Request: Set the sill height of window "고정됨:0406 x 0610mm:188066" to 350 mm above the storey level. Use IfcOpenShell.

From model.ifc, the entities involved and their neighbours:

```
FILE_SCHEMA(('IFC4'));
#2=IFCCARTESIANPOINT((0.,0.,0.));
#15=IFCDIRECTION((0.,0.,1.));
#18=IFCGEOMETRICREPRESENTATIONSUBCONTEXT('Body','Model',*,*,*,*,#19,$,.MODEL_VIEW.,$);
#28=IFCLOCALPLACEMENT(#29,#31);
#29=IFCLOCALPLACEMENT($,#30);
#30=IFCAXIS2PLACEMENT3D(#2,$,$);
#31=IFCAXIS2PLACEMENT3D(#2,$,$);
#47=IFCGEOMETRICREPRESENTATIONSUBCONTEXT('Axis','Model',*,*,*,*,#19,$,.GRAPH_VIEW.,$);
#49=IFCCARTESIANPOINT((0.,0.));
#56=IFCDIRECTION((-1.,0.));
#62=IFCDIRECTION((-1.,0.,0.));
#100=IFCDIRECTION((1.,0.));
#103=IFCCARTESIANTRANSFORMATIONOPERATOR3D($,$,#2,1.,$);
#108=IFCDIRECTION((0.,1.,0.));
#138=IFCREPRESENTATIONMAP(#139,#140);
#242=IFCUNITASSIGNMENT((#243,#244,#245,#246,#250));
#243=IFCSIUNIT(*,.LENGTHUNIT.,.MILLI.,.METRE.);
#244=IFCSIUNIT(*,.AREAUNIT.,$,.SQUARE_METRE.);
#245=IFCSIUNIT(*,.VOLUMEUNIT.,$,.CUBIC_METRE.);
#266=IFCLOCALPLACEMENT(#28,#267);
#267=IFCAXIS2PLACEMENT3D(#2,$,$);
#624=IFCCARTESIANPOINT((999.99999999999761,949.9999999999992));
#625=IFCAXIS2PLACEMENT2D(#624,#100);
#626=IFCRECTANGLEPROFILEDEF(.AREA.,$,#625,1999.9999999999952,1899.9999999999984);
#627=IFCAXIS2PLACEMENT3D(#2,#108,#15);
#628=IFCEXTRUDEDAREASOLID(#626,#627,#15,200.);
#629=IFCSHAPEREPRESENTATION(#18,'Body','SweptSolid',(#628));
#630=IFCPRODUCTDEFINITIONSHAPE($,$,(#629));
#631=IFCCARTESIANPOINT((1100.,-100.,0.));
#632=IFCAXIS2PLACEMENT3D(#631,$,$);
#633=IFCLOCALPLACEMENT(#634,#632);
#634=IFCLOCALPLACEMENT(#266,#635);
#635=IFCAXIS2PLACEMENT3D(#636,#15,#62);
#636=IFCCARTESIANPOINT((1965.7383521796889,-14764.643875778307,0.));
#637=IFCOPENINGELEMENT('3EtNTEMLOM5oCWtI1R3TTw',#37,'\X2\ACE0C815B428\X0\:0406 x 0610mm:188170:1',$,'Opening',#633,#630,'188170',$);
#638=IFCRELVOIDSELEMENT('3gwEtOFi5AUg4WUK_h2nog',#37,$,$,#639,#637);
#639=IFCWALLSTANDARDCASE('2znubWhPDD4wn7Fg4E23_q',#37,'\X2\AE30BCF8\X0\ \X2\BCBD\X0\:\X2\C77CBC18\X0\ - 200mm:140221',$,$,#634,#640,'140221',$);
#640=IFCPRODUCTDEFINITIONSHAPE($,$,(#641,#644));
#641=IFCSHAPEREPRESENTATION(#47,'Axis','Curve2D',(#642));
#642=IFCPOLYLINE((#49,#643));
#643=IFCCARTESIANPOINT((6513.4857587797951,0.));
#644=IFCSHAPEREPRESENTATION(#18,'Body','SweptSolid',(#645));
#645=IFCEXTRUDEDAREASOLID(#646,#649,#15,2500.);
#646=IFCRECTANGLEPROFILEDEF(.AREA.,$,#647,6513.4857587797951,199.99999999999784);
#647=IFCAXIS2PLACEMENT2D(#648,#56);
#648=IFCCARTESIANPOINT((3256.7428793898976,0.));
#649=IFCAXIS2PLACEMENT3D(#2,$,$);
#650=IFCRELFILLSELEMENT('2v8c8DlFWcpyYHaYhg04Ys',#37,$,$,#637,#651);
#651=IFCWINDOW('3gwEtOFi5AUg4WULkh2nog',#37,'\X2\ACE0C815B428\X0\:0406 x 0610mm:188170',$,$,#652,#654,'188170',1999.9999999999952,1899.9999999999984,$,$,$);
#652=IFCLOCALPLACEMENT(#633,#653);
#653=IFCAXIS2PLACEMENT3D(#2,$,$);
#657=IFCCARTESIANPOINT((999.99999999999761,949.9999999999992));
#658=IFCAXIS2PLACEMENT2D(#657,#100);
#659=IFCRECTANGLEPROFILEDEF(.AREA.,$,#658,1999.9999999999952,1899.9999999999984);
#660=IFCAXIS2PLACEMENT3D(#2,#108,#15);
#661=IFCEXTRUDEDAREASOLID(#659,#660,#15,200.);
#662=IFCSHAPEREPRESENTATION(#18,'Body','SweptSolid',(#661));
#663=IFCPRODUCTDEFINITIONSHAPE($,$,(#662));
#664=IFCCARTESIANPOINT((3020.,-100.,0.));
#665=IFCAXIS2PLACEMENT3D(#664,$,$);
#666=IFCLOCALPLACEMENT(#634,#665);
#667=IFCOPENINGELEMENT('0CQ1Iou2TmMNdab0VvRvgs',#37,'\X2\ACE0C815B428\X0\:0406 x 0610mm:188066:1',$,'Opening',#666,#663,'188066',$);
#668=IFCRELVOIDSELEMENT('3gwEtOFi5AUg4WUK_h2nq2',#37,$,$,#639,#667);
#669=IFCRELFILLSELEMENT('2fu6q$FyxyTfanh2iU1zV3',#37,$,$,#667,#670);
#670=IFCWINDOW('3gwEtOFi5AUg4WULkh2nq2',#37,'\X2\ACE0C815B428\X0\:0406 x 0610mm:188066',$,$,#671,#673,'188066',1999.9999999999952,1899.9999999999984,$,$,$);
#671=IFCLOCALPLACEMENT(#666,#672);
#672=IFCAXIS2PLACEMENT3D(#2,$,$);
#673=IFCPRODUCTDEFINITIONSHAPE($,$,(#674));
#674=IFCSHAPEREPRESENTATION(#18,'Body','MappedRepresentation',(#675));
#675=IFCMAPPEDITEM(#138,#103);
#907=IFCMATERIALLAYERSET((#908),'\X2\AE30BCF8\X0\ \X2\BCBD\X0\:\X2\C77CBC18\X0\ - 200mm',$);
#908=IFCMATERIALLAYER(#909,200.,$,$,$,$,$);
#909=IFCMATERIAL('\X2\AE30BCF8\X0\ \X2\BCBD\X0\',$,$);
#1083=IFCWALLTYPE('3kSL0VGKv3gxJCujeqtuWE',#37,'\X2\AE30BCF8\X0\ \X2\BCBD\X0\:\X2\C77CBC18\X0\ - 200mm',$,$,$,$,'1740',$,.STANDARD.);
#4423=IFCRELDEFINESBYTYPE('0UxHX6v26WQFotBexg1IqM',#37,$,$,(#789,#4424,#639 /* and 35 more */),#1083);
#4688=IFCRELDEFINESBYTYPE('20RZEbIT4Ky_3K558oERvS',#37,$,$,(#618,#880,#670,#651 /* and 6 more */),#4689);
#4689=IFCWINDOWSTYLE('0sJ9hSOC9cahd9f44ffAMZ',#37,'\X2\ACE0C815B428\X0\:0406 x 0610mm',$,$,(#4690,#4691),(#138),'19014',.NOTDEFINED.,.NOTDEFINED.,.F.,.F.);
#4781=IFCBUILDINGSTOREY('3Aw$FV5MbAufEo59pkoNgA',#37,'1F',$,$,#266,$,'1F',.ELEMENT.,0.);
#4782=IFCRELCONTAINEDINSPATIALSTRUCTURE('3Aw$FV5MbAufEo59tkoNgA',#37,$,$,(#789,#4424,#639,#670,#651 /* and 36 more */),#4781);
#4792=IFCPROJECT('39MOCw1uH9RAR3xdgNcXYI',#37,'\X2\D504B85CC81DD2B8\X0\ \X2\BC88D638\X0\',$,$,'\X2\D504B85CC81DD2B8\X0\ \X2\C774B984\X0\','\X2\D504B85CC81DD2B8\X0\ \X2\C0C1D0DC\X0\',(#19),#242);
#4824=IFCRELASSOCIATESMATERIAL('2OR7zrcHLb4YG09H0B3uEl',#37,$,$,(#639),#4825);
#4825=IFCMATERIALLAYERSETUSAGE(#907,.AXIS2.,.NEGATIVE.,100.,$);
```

```python
import numpy as np
import ifcopenshell
import ifcopenshell.api.geometry
import ifcopenshell.geom
import ifcopenshell.util.element
import ifcopenshell.util.placement
import ifcopenshell.util.shape
import ifcopenshell.util.unit

model = ifcopenshell.open("model.ifc")
unit_scale = ifcopenshell.util.unit.calculate_unit_scale(model)

window = model.by_guid("3gwEtOFi5AUg4WULkh2nq2")
opening = window.FillsVoids[0].RelatingOpeningElement
storey = ifcopenshell.util.element.get_container(window, ifc_class="IfcBuildingStorey")
level = ifcopenshell.util.placement.get_local_placement(storey.ObjectPlacement)[2, 3]

# The opening's origin need not be at the sill, so measure its lowest point.
shape = ifcopenshell.geom.create_shape(ifcopenshell.geom.settings(), opening)
bottom = ifcopenshell.util.shape.get_shape_bottom_elevation(shape, shape.geometry) / unit_scale
dz = level + 0.35 / unit_scale - bottom

shift = np.array([0.0, 0.0, dz])
# The window is placed relative to its opening, so it follows when the opening moves.
matrix = ifcopenshell.util.placement.get_local_placement(opening.ObjectPlacement)
matrix[:3, 3] += shift
ifcopenshell.api.geometry.edit_object_placement(
    model, product=opening, matrix=matrix, is_si=False, should_transform_children=True
)

print(f"moved by {dz * unit_scale:+.3f} m")

model.write("model_updated.ifc")
```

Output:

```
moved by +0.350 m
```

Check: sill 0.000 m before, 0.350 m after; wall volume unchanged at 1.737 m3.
